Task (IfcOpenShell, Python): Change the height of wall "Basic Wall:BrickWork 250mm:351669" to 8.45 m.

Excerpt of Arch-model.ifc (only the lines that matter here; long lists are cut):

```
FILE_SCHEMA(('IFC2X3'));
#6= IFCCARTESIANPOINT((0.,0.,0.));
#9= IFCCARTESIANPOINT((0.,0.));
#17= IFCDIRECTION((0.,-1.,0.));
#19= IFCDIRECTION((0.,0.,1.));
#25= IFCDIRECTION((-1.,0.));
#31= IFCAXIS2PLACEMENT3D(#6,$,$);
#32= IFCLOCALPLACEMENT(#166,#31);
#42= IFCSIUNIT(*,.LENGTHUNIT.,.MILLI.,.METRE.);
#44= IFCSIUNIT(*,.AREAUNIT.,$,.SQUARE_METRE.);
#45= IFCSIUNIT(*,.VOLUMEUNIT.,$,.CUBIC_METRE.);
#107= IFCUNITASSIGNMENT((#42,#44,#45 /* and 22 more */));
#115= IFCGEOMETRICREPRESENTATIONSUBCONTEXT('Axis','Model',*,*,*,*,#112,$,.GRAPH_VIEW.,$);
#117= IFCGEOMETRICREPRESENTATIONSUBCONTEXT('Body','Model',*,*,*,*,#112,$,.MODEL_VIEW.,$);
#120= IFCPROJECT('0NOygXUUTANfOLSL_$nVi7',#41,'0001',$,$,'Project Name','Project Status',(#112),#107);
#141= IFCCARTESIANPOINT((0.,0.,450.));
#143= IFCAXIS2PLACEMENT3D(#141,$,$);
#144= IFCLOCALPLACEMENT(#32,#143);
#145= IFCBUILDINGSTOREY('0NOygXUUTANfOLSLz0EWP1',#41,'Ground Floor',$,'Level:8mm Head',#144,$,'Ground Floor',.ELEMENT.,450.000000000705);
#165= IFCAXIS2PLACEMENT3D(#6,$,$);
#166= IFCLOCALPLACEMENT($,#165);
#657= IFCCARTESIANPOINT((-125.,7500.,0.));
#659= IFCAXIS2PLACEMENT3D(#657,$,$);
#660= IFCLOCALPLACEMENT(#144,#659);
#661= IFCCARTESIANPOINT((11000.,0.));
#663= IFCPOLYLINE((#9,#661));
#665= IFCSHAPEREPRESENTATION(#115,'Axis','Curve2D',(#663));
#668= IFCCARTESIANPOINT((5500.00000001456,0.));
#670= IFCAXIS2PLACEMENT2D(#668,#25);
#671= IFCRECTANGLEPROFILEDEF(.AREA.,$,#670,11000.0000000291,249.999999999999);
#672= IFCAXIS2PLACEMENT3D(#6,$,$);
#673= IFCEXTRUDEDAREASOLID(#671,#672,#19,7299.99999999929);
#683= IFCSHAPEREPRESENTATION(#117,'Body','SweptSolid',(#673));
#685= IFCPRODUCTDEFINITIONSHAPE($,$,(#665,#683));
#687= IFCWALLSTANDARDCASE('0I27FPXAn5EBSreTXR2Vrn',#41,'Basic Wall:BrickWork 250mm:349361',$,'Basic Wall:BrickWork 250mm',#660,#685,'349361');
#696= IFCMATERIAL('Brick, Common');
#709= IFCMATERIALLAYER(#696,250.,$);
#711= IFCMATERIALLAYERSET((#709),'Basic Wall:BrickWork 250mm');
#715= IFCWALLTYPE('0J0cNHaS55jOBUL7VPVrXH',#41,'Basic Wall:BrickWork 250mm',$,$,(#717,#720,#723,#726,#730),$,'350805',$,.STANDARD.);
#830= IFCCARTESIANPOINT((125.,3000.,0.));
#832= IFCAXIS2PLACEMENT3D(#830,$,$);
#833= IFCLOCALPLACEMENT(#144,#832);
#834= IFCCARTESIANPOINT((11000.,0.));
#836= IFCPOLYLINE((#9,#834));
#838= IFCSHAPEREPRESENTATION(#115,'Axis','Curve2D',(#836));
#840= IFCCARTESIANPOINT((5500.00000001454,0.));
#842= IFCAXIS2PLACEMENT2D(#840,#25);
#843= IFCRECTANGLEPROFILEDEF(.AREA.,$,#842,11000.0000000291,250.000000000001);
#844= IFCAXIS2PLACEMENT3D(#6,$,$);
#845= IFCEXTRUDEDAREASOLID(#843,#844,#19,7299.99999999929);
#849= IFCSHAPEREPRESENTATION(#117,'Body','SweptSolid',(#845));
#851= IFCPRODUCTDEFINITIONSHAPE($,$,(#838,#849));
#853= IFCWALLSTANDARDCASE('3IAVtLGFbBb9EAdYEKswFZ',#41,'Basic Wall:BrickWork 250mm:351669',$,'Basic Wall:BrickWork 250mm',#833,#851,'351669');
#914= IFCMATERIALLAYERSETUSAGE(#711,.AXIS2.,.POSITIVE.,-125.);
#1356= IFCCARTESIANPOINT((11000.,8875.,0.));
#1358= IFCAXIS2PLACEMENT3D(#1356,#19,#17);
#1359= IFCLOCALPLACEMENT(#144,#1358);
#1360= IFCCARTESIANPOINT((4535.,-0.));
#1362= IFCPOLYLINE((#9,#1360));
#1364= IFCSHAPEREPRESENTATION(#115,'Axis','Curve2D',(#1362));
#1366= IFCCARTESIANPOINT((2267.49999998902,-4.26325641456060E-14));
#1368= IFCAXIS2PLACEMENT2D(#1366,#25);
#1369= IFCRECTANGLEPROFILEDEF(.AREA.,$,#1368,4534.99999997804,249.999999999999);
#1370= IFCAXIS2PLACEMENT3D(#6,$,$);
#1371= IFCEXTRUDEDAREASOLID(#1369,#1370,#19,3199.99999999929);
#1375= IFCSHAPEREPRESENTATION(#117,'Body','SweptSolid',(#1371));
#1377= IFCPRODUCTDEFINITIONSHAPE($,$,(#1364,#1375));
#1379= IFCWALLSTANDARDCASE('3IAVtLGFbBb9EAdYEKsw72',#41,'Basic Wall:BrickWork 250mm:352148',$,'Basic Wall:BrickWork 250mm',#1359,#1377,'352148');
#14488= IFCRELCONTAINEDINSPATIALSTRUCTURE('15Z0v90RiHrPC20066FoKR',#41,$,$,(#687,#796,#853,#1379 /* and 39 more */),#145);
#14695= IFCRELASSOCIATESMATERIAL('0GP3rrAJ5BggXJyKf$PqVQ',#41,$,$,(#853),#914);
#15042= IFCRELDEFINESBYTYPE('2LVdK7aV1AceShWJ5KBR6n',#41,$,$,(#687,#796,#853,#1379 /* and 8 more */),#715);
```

```python
import ifcopenshell
import ifcopenshell.geom
import ifcopenshell.util.representation
import ifcopenshell.util.shape

model = ifcopenshell.open("Arch-model.ifc")
settings = ifcopenshell.geom.settings()


def volume(element):
    """Net volume in cubic metres, openings subtracted."""
    shape = ifcopenshell.geom.create_shape(settings, element)
    return ifcopenshell.util.shape.get_volume(shape.geometry)


wall = model.by_guid("3IAVtLGFbBb9EAdYEKswFZ")
before = volume(wall)

body = ifcopenshell.util.representation.get_representation(wall, "Model", "Body")
solid = body.Items[0]
old_height = solid.Depth
solid.Depth = 8450.0
after = volume(wall)

print(f"height {old_height:g} -> {solid.Depth:g}, volume {before:.3f} -> {after:.3f} m3")

model.write("Arch-model_rev.ifc")
```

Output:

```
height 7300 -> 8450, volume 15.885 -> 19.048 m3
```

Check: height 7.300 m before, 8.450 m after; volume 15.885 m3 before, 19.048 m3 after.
